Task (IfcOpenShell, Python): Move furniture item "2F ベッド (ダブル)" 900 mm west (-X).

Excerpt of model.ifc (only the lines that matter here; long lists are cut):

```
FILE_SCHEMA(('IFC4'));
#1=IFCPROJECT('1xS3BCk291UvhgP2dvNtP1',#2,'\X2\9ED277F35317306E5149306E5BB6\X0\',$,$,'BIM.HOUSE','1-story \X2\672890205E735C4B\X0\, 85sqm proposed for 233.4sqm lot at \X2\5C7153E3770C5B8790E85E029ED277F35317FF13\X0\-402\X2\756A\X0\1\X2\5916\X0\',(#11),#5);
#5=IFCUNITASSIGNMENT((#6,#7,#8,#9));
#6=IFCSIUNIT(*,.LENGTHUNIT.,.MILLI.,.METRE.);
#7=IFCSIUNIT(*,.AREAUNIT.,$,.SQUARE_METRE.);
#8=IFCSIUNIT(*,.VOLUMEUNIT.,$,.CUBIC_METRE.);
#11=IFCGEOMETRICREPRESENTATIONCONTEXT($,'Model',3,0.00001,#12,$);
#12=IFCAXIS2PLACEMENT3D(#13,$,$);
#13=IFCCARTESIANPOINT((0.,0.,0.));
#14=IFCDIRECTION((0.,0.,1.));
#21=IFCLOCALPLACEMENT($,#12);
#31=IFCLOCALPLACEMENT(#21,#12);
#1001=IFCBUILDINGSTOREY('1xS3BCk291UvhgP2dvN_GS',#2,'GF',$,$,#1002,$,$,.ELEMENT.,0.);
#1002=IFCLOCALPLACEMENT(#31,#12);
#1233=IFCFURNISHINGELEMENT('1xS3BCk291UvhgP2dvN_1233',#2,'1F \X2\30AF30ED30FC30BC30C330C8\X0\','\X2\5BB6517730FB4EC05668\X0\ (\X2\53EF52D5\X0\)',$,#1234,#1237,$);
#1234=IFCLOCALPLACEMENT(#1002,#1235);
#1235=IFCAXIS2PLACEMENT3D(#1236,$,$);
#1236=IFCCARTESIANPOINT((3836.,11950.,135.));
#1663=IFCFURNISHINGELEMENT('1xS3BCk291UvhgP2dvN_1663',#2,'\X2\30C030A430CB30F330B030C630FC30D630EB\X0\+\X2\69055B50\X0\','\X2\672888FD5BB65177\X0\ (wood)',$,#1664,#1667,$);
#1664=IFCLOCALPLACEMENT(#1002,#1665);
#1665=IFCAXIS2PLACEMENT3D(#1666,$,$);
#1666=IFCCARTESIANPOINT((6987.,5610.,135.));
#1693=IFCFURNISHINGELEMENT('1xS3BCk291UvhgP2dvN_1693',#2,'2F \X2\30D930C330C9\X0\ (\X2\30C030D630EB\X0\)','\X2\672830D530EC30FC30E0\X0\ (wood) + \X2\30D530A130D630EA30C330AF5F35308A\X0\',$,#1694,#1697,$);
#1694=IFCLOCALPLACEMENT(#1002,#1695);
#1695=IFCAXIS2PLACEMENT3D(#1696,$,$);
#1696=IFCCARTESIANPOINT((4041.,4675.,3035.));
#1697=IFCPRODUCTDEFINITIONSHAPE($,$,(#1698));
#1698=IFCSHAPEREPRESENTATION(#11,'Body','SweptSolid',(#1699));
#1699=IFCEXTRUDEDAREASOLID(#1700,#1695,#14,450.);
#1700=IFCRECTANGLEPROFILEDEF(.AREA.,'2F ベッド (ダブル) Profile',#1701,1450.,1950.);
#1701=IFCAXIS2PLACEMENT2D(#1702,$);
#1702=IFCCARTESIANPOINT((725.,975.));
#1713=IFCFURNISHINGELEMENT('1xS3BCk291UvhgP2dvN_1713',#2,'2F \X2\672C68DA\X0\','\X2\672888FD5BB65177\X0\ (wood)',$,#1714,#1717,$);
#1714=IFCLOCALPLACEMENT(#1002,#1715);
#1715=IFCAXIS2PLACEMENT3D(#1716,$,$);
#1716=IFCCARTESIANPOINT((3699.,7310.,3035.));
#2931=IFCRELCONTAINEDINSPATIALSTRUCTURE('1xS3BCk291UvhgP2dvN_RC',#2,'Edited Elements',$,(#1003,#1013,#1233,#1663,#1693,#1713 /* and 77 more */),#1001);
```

```python
import ifcopenshell
import ifcopenshell.api.geometry
import ifcopenshell.util.placement
import ifcopenshell.util.unit

model = ifcopenshell.open("model.ifc")
unit_scale = ifcopenshell.util.unit.calculate_unit_scale(model)

item = model.by_guid("1xS3BCk291UvhgP2dvN_1693")
matrix = ifcopenshell.util.placement.get_local_placement(item.ObjectPlacement)
matrix[0, 3] -= 0.9 / unit_scale
ifcopenshell.api.geometry.edit_object_placement(model, product=item, matrix=matrix, is_si=False)

print(ifcopenshell.util.placement.get_local_placement(item.ObjectPlacement).round(3) + 0.0)

model.write("model-out.ifc")
```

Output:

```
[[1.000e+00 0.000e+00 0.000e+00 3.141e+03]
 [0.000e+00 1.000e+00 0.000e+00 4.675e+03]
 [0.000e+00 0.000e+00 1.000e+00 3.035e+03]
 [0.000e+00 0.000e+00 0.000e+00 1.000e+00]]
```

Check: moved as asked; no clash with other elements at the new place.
